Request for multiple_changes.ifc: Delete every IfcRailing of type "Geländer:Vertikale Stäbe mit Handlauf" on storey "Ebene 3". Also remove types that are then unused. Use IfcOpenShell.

First a look at what the model holds.

```python
import ifcopenshell
import ifcopenshell.util.element

model = ifcopenshell.open("multiple_changes.ifc")
print(model.schema)
storey = next(s for s in model.by_type("IfcBuildingStorey") if s.Name == "Ebene 3")
railings = [e for e in ifcopenshell.util.element.get_decomposition(storey) if e.is_a("IfcRailing")]
seen = {}
for e in railings:
    element_type = ifcopenshell.util.element.get_type(e)
    name = element_type.Name if element_type not in (None, e) else None
    seen[name] = seen.get(name, 0) + 1
for name, count in sorted(seen.items(), key=str):
    print(count, "x", name)
```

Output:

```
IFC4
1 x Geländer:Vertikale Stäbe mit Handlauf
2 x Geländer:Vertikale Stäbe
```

```python
import ifcopenshell
import ifcopenshell.api.root
import ifcopenshell.util.element

model = ifcopenshell.open("multiple_changes.ifc")

storey = next(s for s in model.by_type("IfcBuildingStorey") if s.Name == "Ebene 3")
railings = [e for e in ifcopenshell.util.element.get_decomposition(storey) if e.is_a("IfcRailing")]
targets = [e for e in railings if (t := ifcopenshell.util.element.get_type(e)) not in (None, e) and t.Name == "Geländer:Vertikale Stäbe mit Handlauf"]
types = {ifcopenshell.util.element.get_type(e) for e in targets} - {None, *targets}

for e in targets:
    ifcopenshell.api.root.remove_product(model, product=e)
print(len(targets), "removed")

unused = [t for t in types if not ifcopenshell.util.element.get_types(t)]
for t in unused:
    ifcopenshell.api.root.remove_product(model, product=t)
print(len(unused), "unused types removed")

model.write("multiple_changes_v2.ifc")
```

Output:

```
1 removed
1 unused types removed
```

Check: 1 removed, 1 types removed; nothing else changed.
